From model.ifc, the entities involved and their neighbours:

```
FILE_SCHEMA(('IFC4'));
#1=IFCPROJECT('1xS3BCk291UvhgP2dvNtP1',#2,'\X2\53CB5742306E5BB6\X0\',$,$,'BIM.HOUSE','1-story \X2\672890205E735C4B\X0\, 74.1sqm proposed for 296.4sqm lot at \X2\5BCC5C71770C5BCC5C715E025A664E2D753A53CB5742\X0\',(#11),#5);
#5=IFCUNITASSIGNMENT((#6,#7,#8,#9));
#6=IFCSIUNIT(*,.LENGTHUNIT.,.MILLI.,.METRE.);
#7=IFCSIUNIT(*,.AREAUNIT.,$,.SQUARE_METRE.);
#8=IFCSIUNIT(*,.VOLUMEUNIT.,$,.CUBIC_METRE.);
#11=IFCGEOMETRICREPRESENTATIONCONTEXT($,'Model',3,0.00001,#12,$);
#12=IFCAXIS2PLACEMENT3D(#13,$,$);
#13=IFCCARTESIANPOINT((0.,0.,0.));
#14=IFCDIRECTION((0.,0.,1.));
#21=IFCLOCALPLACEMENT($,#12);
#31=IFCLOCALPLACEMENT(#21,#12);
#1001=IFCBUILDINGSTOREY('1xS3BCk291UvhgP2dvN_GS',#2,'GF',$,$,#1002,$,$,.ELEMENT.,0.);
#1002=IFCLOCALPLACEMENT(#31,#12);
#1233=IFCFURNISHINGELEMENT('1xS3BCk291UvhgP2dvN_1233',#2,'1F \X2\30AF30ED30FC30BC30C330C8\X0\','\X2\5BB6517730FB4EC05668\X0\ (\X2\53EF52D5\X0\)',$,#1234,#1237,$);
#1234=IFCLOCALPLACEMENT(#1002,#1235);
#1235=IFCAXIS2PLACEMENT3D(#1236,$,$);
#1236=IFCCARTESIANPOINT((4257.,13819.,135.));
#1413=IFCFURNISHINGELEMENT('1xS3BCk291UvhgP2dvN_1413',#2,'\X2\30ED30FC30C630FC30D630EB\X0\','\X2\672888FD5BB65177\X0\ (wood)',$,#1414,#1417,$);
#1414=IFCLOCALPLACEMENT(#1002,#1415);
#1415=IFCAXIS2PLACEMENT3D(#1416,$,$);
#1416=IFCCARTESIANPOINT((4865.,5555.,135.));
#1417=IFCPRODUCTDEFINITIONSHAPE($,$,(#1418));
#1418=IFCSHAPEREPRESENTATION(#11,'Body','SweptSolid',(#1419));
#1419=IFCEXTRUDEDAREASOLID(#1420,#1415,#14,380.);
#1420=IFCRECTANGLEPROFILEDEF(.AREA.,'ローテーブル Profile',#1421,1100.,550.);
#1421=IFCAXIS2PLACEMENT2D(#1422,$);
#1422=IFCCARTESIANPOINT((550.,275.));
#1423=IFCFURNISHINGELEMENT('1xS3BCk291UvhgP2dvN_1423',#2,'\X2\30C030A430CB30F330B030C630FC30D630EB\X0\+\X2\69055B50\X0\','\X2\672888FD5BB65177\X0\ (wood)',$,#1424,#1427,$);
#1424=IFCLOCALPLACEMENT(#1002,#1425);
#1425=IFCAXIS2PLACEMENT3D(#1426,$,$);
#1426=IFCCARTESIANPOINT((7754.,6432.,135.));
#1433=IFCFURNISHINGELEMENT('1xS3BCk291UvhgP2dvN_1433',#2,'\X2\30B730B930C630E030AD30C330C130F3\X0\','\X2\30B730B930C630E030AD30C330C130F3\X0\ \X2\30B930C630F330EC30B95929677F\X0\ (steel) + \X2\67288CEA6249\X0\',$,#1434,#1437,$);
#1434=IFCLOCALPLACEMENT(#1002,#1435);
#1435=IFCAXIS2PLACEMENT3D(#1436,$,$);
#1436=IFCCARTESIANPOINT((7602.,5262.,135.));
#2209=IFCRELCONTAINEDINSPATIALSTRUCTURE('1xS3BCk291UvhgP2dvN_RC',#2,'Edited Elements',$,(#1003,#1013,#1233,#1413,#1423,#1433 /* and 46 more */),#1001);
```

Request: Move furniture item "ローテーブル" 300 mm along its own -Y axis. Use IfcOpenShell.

```python
import ifcopenshell
import ifcopenshell.api.geometry
import ifcopenshell.util.placement
import ifcopenshell.util.unit

model = ifcopenshell.open("model.ifc")
unit_scale = ifcopenshell.util.unit.calculate_unit_scale(model)

item = model.by_id(1413)
matrix = ifcopenshell.util.placement.get_local_placement(item.ObjectPlacement)
matrix[:3, 3] -= matrix[:3, 1] * 0.3 / unit_scale
ifcopenshell.api.geometry.edit_object_placement(model, product=item, matrix=matrix, is_si=False)

print(ifcopenshell.util.placement.get_local_placement(item.ObjectPlacement).round(3) + 0.0)

model.write("model_v2.ifc")
```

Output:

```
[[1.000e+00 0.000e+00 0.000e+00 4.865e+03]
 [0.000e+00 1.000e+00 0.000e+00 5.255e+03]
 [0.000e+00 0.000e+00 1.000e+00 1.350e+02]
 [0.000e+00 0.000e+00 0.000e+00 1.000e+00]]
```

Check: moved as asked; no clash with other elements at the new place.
